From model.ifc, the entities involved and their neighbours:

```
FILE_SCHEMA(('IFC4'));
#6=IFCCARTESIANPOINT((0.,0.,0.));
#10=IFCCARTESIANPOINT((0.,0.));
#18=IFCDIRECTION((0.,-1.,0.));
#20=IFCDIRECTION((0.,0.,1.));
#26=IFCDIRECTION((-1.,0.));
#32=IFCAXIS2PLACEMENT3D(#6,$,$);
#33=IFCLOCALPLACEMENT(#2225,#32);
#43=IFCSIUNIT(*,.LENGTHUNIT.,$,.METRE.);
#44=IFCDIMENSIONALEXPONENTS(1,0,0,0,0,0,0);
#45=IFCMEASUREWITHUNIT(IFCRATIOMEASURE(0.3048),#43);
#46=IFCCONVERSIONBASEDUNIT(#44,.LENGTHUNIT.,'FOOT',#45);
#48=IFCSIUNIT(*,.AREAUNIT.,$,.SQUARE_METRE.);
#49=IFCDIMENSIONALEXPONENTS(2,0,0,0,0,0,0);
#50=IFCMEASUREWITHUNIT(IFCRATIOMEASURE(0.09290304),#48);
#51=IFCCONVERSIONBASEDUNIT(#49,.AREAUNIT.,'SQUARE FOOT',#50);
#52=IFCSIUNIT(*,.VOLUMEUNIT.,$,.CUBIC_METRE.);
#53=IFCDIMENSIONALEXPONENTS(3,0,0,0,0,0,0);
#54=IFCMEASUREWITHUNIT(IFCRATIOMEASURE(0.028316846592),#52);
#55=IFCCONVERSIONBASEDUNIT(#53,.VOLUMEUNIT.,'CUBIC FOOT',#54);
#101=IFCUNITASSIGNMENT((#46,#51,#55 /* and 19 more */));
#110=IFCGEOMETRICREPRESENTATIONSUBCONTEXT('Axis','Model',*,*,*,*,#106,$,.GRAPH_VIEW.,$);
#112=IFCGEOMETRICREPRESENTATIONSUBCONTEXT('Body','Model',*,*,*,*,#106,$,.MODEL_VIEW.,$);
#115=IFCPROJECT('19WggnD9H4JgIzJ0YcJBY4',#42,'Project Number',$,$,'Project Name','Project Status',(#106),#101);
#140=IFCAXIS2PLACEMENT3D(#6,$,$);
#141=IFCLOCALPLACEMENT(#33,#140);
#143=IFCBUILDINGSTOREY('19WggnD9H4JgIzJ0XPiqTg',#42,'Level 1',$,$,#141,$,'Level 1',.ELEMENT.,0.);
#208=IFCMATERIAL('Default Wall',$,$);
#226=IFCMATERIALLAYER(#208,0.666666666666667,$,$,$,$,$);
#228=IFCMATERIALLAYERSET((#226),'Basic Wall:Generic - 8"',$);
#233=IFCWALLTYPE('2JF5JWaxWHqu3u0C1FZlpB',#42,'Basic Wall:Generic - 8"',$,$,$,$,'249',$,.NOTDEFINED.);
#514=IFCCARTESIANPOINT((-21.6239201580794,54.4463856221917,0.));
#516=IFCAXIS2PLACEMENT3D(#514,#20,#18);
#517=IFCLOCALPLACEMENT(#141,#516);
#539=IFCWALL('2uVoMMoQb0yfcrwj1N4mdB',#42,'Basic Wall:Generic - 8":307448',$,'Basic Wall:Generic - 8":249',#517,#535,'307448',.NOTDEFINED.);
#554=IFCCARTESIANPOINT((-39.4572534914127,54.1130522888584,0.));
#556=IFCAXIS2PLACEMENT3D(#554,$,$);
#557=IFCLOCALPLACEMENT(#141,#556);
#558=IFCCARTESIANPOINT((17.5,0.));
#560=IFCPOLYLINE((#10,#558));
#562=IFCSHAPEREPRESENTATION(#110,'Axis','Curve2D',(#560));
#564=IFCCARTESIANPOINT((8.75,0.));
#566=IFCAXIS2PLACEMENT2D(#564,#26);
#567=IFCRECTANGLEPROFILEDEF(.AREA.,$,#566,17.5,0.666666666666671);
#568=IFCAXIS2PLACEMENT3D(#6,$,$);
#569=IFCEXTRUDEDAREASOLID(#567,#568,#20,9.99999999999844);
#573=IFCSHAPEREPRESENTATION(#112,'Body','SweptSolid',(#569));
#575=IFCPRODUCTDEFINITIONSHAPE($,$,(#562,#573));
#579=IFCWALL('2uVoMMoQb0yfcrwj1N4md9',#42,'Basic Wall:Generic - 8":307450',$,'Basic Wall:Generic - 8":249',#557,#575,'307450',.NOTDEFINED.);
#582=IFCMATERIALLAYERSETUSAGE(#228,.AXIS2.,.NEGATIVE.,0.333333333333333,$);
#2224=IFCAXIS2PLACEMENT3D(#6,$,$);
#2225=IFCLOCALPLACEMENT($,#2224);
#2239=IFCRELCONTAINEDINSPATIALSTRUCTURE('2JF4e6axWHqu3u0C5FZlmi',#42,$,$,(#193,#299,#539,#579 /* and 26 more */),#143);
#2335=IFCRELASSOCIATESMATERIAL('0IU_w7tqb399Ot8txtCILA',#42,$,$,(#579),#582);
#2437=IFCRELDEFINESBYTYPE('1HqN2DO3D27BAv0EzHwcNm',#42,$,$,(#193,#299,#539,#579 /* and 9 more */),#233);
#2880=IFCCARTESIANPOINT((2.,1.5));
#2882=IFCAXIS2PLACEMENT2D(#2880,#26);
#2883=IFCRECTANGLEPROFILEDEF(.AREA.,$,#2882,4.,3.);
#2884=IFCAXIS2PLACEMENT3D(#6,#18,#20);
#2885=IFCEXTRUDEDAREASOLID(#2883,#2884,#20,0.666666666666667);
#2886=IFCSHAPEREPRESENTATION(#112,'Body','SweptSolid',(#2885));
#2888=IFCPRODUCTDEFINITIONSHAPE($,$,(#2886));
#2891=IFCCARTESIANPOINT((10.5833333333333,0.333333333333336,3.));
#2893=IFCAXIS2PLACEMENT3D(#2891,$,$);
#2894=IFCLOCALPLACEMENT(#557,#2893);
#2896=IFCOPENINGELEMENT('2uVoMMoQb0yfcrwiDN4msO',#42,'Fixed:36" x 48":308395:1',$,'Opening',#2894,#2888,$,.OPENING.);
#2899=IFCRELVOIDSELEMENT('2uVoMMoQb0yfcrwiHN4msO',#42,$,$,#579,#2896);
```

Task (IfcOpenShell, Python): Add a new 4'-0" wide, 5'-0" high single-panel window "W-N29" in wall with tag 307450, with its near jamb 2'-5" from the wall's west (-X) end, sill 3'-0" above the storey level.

```python
import numpy as np
import ifcopenshell
import ifcopenshell.api.feature
import ifcopenshell.api.geometry
import ifcopenshell.api.root
import ifcopenshell.api.spatial
import ifcopenshell.geom
import ifcopenshell.util.element
import ifcopenshell.util.placement
import ifcopenshell.util.representation
import ifcopenshell.util.shape
import ifcopenshell.util.unit

model = ifcopenshell.open("model.ifc")
unit_scale = ifcopenshell.util.unit.calculate_unit_scale(model)
settings = ifcopenshell.geom.settings()


def volume(element):
    """Net volume in cubic metres, openings subtracted."""
    shape = ifcopenshell.geom.create_shape(settings, element)
    return ifcopenshell.util.shape.get_volume(shape.geometry)


wall = model.by_guid("2uVoMMoQb0yfcrwj1N4md9")
storey = ifcopenshell.util.element.get_container(wall, ifc_class="IfcBuildingStorey")
context = ifcopenshell.util.representation.get_context(model, "Model", "Body", "MODEL_VIEW")
before = volume(wall)

width, height, from_end, sill = 1.2192, 1.524, 0.7366, 0.9144  # metres

# The wall runs along its own X axis, and the end named is its -X end.
wall_shape = ifcopenshell.geom.create_shape(settings, wall)
x, y, z = ifcopenshell.util.shape.get_vertices(wall_shape.geometry).T
start = x.min() + from_end
face, thickness = float(y.min()), float(y.max() - y.min())
wall_matrix = ifcopenshell.util.placement.get_local_placement(wall.ObjectPlacement)
level = ifcopenshell.util.placement.get_local_placement(storey.ObjectPlacement)[2, 3]


def in_wall(x, y):
    """Placement at x, y metres in the wall's axes, at sill height."""
    matrix = wall_matrix.copy()
    matrix[:, 3] = wall_matrix @ np.array([x / unit_scale, y / unit_scale, 0.0, 1.0])
    matrix[2, 3] = level + sill / unit_scale
    return matrix


# Opening: a box that overshoots both wall faces by 50 mm.
opening = ifcopenshell.api.root.create_entity(model, ifc_class="IfcOpeningElement", predefined_type="OPENING")
box = ifcopenshell.api.geometry.add_wall_representation(
    model, context=context, length=width, height=height, thickness=thickness + 0.1
)
ifcopenshell.api.geometry.assign_representation(model, product=opening, representation=box)
ifcopenshell.api.geometry.edit_object_placement(model, product=opening, matrix=in_wall(start, face - 0.05), is_si=False)
ifcopenshell.api.feature.add_feature(model, feature=opening, element=wall)

window = ifcopenshell.api.root.create_entity(model, ifc_class="IfcWindow", name="W-N29", predefined_type="WINDOW")
window.OverallWidth, window.OverallHeight = width / unit_scale, height / unit_scale
window.PartitioningType = "SINGLE_PANEL"
body = ifcopenshell.api.geometry.add_window_representation(
    model,
    context=context,
    overall_width=window.OverallWidth,
    overall_height=window.OverallHeight,
    partition_type="SINGLE_PANEL",
)
ifcopenshell.api.geometry.assign_representation(model, product=window, representation=body)
ifcopenshell.api.spatial.assign_container(model, products=[window], relating_structure=storey)
ifcopenshell.api.feature.add_filling(model, opening=opening, element=window)

# Centre the window in the wall's thickness.
ifcopenshell.api.geometry.edit_object_placement(model, product=window, matrix=in_wall(start, face), is_si=False)
window_shape = ifcopenshell.geom.create_shape(settings, window)
depth = ifcopenshell.util.shape.get_vertices(window_shape.geometry)[:, 1]
offset = face + thickness / 2 - (depth.min() + depth.max()) / 2
ifcopenshell.api.geometry.edit_object_placement(model, product=window, matrix=in_wall(start, offset), is_si=False)

after = volume(wall)

print(f"wall volume {before:.3f} -> {after:.3f} m3")

model.write("model_v2.ifc")
```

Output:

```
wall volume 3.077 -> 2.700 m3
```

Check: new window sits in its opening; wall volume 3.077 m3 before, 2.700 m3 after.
